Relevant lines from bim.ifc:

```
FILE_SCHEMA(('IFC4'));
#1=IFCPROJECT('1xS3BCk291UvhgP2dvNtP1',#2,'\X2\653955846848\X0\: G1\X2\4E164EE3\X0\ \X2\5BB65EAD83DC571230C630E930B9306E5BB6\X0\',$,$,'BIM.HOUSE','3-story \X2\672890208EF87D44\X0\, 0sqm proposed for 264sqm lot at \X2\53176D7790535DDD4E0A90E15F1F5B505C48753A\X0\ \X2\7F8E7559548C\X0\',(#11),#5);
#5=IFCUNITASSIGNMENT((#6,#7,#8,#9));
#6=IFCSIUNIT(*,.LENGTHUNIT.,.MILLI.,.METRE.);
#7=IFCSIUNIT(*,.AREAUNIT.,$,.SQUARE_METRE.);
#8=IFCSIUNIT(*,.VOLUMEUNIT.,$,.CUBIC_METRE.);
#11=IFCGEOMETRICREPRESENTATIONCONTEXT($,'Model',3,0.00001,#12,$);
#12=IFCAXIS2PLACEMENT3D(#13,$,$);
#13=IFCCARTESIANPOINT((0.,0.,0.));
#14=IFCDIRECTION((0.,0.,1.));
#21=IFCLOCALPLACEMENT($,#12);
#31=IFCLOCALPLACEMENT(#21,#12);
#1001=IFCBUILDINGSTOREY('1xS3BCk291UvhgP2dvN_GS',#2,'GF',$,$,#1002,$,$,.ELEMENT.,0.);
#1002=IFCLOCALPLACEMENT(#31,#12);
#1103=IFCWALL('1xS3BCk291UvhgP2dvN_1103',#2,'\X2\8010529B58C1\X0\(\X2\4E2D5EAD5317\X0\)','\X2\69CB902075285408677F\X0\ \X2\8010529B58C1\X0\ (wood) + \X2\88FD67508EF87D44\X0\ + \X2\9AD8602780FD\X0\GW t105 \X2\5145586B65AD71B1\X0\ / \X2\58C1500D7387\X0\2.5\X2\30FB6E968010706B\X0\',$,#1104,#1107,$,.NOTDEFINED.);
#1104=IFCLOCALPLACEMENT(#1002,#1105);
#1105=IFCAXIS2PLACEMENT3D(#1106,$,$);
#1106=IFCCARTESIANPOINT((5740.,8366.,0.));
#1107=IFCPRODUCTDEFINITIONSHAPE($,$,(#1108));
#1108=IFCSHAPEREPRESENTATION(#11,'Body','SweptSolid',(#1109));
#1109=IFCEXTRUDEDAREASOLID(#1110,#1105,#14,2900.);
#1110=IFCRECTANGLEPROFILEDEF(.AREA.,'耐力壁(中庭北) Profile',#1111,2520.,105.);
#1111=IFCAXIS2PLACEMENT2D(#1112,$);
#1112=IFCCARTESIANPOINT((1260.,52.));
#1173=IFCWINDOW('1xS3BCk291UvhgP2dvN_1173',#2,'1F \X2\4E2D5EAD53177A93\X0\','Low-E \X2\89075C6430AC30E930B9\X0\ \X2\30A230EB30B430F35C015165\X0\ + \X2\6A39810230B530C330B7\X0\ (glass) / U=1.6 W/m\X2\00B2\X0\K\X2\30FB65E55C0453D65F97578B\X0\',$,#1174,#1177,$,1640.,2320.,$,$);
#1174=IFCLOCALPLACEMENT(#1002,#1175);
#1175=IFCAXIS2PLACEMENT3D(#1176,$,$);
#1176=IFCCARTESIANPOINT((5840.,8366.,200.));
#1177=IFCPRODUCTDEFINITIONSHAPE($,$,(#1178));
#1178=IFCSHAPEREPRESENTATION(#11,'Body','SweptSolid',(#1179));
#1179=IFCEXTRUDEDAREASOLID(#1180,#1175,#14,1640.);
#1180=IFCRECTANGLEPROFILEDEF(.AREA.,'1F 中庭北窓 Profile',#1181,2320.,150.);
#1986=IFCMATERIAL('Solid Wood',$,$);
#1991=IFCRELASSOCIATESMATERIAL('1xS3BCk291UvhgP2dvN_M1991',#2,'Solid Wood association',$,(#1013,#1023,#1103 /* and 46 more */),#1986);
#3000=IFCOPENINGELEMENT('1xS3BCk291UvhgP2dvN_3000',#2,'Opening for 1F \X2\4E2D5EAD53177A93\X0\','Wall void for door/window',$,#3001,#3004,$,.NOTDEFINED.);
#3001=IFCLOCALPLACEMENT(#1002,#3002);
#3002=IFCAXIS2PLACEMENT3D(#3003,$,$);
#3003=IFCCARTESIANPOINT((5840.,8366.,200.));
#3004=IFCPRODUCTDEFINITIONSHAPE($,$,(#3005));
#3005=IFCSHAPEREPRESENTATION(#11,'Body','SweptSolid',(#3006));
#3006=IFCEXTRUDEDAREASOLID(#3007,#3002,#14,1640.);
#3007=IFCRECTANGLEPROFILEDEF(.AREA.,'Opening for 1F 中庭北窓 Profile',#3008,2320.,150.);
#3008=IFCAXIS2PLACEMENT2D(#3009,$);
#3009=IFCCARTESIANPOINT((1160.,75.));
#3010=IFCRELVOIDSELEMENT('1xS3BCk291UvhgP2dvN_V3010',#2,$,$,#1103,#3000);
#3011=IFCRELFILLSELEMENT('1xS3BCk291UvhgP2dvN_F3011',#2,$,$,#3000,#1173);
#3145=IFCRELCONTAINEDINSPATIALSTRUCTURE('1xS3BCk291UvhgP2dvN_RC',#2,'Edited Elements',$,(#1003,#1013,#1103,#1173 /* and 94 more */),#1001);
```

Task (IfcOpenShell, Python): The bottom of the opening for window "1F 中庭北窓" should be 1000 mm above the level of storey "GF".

```python
import numpy as np
import ifcopenshell
import ifcopenshell.api.geometry
import ifcopenshell.geom
import ifcopenshell.util.element
import ifcopenshell.util.placement
import ifcopenshell.util.shape
import ifcopenshell.util.unit

model = ifcopenshell.open("bim.ifc")
unit_scale = ifcopenshell.util.unit.calculate_unit_scale(model)

window = model.by_guid("1xS3BCk291UvhgP2dvN_1173")
opening = window.FillsVoids[0].RelatingOpeningElement
storey = ifcopenshell.util.element.get_container(window, ifc_class="IfcBuildingStorey")
level = ifcopenshell.util.placement.get_local_placement(storey.ObjectPlacement)[2, 3]

# The opening's origin need not be at the sill, so measure its lowest point.
shape = ifcopenshell.geom.create_shape(ifcopenshell.geom.settings(), opening)
bottom = ifcopenshell.util.shape.get_shape_bottom_elevation(shape, shape.geometry) / unit_scale
dz = level + 1 / unit_scale - bottom

shift = np.array([0.0, 0.0, dz])
# The window is not placed relative to its opening, so move both.
for product in (opening, window):
    matrix = ifcopenshell.util.placement.get_local_placement(product.ObjectPlacement)
    matrix[:3, 3] += shift
    ifcopenshell.api.geometry.edit_object_placement(model, product=product, matrix=matrix, is_si=False)

print(f"moved by {dz * unit_scale:+.3f} m")

model.write("bim_updated.ifc")
```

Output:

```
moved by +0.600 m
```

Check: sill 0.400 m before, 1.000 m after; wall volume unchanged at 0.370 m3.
